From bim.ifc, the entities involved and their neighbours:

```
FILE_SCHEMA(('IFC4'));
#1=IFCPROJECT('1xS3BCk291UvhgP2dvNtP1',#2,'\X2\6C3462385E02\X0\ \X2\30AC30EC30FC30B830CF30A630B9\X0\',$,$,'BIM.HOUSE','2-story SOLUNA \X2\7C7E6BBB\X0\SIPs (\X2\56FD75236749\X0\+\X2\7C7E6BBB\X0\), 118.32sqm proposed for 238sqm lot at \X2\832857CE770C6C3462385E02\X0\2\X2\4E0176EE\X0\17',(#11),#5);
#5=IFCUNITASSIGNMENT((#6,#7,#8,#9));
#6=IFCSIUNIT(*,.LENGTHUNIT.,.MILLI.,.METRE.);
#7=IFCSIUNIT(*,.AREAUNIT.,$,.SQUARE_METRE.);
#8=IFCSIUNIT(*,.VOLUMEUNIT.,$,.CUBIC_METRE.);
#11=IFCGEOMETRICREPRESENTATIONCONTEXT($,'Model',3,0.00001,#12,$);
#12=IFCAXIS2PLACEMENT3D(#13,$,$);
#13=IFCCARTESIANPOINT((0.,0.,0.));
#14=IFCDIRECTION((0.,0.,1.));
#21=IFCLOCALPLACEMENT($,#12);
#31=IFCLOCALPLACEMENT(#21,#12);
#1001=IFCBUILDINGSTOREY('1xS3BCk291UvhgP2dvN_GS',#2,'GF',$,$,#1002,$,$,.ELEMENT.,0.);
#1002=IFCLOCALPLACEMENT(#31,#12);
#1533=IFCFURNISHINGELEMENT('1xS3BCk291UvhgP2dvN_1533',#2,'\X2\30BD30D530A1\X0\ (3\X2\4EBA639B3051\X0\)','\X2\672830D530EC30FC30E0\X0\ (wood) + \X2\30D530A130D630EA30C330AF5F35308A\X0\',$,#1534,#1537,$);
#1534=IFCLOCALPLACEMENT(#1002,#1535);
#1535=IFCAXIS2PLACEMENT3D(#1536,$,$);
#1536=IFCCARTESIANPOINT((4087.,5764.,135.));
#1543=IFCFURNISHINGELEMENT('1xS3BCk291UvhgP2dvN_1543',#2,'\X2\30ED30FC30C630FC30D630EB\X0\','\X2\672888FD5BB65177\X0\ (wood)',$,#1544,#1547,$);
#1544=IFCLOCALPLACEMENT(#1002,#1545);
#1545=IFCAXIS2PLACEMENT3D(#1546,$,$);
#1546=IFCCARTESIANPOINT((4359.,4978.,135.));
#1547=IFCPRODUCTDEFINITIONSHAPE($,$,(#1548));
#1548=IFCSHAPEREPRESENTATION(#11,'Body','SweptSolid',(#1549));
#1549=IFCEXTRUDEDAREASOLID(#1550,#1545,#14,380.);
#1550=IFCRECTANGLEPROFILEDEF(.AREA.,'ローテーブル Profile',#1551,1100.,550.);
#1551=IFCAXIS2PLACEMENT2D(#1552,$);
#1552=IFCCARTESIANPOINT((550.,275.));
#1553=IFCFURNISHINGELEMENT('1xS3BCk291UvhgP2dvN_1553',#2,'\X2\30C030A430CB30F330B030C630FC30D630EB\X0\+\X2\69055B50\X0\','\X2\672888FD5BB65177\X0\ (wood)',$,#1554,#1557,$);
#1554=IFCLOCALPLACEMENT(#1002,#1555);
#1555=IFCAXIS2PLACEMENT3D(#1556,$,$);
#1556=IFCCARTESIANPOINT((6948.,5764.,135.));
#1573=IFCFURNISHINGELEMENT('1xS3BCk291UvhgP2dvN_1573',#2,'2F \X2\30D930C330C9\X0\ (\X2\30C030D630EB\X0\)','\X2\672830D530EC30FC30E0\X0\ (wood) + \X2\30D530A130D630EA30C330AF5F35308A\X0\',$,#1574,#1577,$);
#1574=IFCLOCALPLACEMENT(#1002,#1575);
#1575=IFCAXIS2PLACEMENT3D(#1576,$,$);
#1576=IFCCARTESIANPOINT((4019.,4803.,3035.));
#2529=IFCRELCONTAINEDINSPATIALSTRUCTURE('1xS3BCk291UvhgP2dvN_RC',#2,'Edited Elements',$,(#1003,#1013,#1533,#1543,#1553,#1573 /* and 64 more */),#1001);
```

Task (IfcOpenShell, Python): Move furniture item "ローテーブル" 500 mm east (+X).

```python
import ifcopenshell
import ifcopenshell.api.geometry
import ifcopenshell.util.placement
import ifcopenshell.util.unit

model = ifcopenshell.open("bim.ifc")
unit_scale = ifcopenshell.util.unit.calculate_unit_scale(model)

item = model.by_guid("1xS3BCk291UvhgP2dvN_1543")
matrix = ifcopenshell.util.placement.get_local_placement(item.ObjectPlacement)
matrix[0, 3] += 0.5 / unit_scale
ifcopenshell.api.geometry.edit_object_placement(model, product=item, matrix=matrix, is_si=False)

print(ifcopenshell.util.placement.get_local_placement(item.ObjectPlacement).round(3) + 0.0)

model.write("bim_updated.ifc")
```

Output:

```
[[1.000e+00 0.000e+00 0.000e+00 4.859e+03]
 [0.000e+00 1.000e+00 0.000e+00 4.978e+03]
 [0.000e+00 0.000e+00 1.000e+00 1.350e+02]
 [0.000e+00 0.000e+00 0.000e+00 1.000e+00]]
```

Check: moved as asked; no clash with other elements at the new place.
